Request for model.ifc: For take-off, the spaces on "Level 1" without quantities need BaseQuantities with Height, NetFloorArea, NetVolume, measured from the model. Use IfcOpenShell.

First a look at what the model holds.

```python
import ifcopenshell
import ifcopenshell.util.element
import ifcopenshell.util.unit

model = ifcopenshell.open("model.ifc")
print(model.schema)
for unit_type in ("LENGTHUNIT", "AREAUNIT", "VOLUMEUNIT"):
    print(unit_type, ifcopenshell.util.unit.calculate_unit_scale(model, unit_type))
storey = next(s for s in model.by_type("IfcBuildingStorey") if s.Name == "Level 1")
spaces = [e for e in ifcopenshell.util.element.get_decomposition(storey) if e.is_a("IfcSpace")]
for e in sorted(spaces, key=lambda e: e.id()):
    print(e.id(), e.is_a(), e.Name, list(ifcopenshell.util.element.get_psets(e, qtos_only=True)), sep=" | ")
```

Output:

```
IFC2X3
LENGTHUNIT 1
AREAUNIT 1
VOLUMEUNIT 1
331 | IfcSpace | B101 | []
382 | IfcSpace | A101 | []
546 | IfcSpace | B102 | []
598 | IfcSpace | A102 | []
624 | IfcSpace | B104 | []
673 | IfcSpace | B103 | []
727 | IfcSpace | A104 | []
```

```python
import ifcopenshell
import ifcopenshell.api.pset
import ifcopenshell.geom
import ifcopenshell.util.element
import ifcopenshell.util.shape
import ifcopenshell.util.unit

model = ifcopenshell.open("model.ifc")
unit_scale = ifcopenshell.util.unit.calculate_unit_scale(model)
area_scale = ifcopenshell.util.unit.calculate_unit_scale(model, "AREAUNIT")
volume_scale = ifcopenshell.util.unit.calculate_unit_scale(model, "VOLUMEUNIT")
settings = ifcopenshell.geom.settings()

storey = next(s for s in model.by_type("IfcBuildingStorey") if s.Name == "Level 1")
spaces = [e for e in ifcopenshell.util.element.get_decomposition(storey) if e.is_a("IfcSpace")]

for e in sorted(spaces, key=lambda e: e.id()):
    if ifcopenshell.util.element.get_psets(e, qtos_only=True, should_inherit=False):
        continue
    # Geometry comes back in metres, in the element's own axes.
    shape = ifcopenshell.geom.create_shape(settings, e)
    values = {
        "Height": ifcopenshell.util.shape.get_z(shape.geometry) / unit_scale,
        "NetFloorArea": ifcopenshell.util.shape.get_footprint_area(shape.geometry) / area_scale,
        "NetVolume": ifcopenshell.util.shape.get_volume(shape.geometry) / volume_scale,
    }
    qto = ifcopenshell.api.pset.add_qto(model, product=e, name="BaseQuantities")
    ifcopenshell.api.pset.edit_qto(model, qto=qto, properties=values)
    print(e.id(), {k: round(v, 3) for k, v in values.items()})

model.write("model_rev.ifc")
```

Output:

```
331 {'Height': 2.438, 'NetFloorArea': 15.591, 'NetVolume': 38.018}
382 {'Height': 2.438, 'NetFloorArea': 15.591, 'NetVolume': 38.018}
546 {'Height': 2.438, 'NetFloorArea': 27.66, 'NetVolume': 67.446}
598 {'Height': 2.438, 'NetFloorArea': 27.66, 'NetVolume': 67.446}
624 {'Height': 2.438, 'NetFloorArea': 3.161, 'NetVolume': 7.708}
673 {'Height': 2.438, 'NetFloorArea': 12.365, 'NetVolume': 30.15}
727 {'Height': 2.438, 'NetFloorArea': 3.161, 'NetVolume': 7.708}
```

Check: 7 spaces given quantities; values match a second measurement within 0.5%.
